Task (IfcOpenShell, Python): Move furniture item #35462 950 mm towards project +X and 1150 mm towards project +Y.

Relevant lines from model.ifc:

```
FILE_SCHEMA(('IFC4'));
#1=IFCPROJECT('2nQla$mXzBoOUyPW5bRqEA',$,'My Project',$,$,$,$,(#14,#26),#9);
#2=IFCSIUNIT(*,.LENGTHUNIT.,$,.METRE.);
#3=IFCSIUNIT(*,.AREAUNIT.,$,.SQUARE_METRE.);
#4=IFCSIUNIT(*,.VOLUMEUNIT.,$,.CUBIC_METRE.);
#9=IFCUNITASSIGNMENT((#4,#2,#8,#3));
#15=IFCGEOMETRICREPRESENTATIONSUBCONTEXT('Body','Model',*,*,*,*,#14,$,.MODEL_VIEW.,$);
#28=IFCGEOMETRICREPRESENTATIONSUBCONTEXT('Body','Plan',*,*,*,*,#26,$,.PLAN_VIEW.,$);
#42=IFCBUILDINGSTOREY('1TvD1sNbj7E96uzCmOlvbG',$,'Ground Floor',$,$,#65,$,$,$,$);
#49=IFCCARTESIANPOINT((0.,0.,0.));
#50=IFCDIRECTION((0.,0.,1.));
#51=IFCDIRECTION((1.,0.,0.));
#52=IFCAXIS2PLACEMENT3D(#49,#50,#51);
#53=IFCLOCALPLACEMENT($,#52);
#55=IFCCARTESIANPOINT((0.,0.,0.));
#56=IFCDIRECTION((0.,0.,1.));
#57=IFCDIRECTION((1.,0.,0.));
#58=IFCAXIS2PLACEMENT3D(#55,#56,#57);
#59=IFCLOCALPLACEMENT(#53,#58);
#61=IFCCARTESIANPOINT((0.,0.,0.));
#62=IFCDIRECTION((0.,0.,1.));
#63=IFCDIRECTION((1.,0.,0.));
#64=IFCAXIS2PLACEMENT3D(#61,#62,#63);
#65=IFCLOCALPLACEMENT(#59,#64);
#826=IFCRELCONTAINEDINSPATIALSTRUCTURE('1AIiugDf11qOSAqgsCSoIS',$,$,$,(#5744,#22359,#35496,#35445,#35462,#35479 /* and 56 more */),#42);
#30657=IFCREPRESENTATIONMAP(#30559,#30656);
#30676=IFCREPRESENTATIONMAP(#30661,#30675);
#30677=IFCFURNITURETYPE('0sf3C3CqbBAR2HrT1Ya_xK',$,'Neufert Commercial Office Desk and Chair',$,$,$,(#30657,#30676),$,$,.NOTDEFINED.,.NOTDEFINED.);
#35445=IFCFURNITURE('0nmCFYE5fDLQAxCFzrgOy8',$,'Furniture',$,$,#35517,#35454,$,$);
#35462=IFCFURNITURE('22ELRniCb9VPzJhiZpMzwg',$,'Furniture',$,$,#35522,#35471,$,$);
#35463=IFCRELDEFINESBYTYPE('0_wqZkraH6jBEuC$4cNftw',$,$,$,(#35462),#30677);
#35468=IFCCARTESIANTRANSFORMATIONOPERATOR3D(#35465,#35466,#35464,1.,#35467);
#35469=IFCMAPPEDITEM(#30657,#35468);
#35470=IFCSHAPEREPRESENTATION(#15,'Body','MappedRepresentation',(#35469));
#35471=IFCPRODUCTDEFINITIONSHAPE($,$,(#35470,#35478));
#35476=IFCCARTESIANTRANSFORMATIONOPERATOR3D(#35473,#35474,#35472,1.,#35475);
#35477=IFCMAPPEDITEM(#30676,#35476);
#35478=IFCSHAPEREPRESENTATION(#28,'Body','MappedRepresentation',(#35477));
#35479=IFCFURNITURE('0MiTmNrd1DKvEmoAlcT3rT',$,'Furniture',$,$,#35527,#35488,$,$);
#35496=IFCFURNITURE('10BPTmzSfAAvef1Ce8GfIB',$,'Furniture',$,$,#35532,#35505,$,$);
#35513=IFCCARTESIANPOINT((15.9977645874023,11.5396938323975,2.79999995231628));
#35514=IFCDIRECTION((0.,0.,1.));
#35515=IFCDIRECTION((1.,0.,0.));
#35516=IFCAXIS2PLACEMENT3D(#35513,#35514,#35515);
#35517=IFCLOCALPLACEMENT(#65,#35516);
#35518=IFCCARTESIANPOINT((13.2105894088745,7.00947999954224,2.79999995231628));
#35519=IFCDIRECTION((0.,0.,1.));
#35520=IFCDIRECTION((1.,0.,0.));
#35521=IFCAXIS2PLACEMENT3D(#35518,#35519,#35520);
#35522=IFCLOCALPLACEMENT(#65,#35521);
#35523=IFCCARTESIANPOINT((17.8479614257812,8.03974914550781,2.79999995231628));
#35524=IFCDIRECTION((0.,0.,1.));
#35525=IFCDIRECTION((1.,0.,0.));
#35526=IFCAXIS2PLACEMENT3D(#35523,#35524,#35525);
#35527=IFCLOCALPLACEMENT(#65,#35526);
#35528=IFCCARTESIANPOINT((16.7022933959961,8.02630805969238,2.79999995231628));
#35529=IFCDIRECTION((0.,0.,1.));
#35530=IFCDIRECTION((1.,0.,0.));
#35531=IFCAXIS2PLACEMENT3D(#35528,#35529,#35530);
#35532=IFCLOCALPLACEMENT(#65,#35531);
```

```python
import ifcopenshell
import ifcopenshell.api.geometry
import ifcopenshell.util.placement

model = ifcopenshell.open("model.ifc")

item = model.by_guid("22ELRniCb9VPzJhiZpMzwg")
matrix = ifcopenshell.util.placement.get_local_placement(item.ObjectPlacement)
matrix[0, 3] += 0.95
matrix[1, 3] += 1.15
ifcopenshell.api.geometry.edit_object_placement(model, product=item, matrix=matrix, is_si=False)

print(ifcopenshell.util.placement.get_local_placement(item.ObjectPlacement).round(3) + 0.0)

model.write("model_updated.ifc")
```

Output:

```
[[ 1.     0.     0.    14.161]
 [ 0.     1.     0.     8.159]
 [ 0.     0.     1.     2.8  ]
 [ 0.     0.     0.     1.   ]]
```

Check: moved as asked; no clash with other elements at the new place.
